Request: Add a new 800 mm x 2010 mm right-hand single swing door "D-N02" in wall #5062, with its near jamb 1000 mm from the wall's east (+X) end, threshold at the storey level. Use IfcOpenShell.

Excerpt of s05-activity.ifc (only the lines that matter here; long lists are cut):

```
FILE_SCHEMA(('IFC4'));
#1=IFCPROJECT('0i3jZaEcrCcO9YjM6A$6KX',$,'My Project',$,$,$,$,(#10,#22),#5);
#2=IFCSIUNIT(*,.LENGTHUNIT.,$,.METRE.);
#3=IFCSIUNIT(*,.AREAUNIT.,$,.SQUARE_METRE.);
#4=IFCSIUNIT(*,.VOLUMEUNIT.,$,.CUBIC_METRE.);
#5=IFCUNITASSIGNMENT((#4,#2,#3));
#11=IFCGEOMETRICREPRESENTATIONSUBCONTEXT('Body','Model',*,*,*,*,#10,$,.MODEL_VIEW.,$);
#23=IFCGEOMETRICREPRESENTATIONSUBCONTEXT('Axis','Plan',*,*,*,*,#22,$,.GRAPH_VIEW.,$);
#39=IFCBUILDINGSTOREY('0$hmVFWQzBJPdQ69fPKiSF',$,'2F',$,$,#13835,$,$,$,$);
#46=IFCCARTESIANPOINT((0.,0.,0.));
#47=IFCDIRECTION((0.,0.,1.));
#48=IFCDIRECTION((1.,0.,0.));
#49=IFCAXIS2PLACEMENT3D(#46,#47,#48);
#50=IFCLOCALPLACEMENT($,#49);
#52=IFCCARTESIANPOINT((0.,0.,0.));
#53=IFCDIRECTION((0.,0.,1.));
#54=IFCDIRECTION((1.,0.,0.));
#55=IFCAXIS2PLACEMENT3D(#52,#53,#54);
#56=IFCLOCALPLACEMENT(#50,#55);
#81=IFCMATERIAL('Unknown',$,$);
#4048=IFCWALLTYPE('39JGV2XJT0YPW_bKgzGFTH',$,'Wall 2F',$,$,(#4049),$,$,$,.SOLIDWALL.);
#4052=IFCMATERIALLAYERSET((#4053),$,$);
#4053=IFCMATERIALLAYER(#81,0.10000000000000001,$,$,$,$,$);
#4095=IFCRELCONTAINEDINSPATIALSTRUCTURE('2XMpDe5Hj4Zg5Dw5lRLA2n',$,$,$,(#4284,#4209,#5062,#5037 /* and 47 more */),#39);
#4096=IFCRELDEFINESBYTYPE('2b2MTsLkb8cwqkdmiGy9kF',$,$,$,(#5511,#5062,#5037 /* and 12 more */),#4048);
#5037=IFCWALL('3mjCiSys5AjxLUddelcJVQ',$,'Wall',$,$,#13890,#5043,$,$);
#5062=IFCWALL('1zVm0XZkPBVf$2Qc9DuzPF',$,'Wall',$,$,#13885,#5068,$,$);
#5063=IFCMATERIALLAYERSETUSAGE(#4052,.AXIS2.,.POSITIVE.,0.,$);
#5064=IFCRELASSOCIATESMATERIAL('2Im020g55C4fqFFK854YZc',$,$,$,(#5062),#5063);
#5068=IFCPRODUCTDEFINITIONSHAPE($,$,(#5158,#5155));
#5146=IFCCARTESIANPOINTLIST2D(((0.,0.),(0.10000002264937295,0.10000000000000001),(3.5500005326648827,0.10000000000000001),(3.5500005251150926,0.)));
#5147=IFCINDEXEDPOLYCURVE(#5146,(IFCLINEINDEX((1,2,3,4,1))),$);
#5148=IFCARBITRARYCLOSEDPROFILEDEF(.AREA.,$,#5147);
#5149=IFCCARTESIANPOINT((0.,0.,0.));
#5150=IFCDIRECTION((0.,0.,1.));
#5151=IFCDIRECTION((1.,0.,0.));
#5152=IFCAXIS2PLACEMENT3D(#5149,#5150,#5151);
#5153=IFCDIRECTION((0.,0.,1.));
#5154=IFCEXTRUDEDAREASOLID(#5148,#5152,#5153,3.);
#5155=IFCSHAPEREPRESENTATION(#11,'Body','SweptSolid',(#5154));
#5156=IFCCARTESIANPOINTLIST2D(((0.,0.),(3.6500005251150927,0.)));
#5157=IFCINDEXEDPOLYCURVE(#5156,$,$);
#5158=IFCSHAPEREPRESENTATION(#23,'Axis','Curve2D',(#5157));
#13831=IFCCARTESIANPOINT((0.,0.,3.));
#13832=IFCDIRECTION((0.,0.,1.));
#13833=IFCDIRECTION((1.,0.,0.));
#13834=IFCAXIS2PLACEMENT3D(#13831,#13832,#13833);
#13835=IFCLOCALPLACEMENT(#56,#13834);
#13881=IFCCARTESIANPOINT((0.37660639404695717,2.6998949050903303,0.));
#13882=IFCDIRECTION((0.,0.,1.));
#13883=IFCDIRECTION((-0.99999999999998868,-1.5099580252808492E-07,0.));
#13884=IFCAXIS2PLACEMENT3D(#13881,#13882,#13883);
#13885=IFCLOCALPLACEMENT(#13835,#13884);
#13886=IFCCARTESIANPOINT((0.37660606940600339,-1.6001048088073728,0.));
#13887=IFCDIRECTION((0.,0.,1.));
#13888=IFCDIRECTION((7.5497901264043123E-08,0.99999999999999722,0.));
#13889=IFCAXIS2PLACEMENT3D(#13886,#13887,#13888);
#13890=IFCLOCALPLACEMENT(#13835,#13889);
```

```python
import numpy as np
import ifcopenshell
import ifcopenshell.api.feature
import ifcopenshell.api.geometry
import ifcopenshell.api.root
import ifcopenshell.api.spatial
import ifcopenshell.geom
import ifcopenshell.util.element
import ifcopenshell.util.placement
import ifcopenshell.util.representation
import ifcopenshell.util.shape
import ifcopenshell.util.unit

model = ifcopenshell.open("s05-activity.ifc")
unit_scale = ifcopenshell.util.unit.calculate_unit_scale(model)
settings = ifcopenshell.geom.settings()


def volume(element):
    """Net volume in cubic metres, openings subtracted."""
    shape = ifcopenshell.geom.create_shape(settings, element)
    return ifcopenshell.util.shape.get_volume(shape.geometry)


wall = model.by_guid("1zVm0XZkPBVf$2Qc9DuzPF")
storey = ifcopenshell.util.element.get_container(wall, ifc_class="IfcBuildingStorey")
context = ifcopenshell.util.representation.get_context(model, "Model", "Body", "MODEL_VIEW")
before = volume(wall)

width, height, from_end, sill = 0.8, 2.01, 1, 0.0  # metres

# The wall runs along its own X axis, and the end named is its -X end.
wall_shape = ifcopenshell.geom.create_shape(settings, wall)
x, y, z = ifcopenshell.util.shape.get_vertices(wall_shape.geometry).T
start = x.min() + from_end
face, thickness = float(y.min()), float(y.max() - y.min())
wall_matrix = ifcopenshell.util.placement.get_local_placement(wall.ObjectPlacement)
level = ifcopenshell.util.placement.get_local_placement(storey.ObjectPlacement)[2, 3]


def in_wall(x, y):
    """Placement at x, y metres in the wall's axes, at sill height."""
    matrix = wall_matrix.copy()
    matrix[:, 3] = wall_matrix @ np.array([x / unit_scale, y / unit_scale, 0.0, 1.0])
    matrix[2, 3] = level + sill / unit_scale
    return matrix


# Opening: a box that overshoots both wall faces by 50 mm.
opening = ifcopenshell.api.root.create_entity(model, ifc_class="IfcOpeningElement", predefined_type="OPENING")
box = ifcopenshell.api.geometry.add_wall_representation(
    model, context=context, length=width, height=height, thickness=thickness + 0.1
)
ifcopenshell.api.geometry.assign_representation(model, product=opening, representation=box)
ifcopenshell.api.geometry.edit_object_placement(model, product=opening, matrix=in_wall(start, face - 0.05), is_si=False)
ifcopenshell.api.feature.add_feature(model, feature=opening, element=wall)

door = ifcopenshell.api.root.create_entity(model, ifc_class="IfcDoor", name="D-N02", predefined_type="DOOR")
door.OverallWidth, door.OverallHeight = width / unit_scale, height / unit_scale
door.OperationType = "SINGLE_SWING_RIGHT"
body = ifcopenshell.api.geometry.add_door_representation(
    model,
    context=context,
    overall_width=door.OverallWidth,
    overall_height=door.OverallHeight,
    operation_type="SINGLE_SWING_RIGHT",
    lining_properties={"LiningDepth": thickness / unit_scale, "ThresholdDepth": thickness / unit_scale},
)
ifcopenshell.api.geometry.assign_representation(model, product=door, representation=body)
ifcopenshell.api.spatial.assign_container(model, products=[door], relating_structure=storey)
ifcopenshell.api.feature.add_filling(model, opening=opening, element=door)

# The lining spans the wall, so the door starts at the wall face.
ifcopenshell.api.geometry.edit_object_placement(model, product=door, matrix=in_wall(start, face), is_si=False)

after = volume(wall)

print(f"wall volume {before:.3f} -> {after:.3f} m3")

model.write("s05-activity-out.ifc")
```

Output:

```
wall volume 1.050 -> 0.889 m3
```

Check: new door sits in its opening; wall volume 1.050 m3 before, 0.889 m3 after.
